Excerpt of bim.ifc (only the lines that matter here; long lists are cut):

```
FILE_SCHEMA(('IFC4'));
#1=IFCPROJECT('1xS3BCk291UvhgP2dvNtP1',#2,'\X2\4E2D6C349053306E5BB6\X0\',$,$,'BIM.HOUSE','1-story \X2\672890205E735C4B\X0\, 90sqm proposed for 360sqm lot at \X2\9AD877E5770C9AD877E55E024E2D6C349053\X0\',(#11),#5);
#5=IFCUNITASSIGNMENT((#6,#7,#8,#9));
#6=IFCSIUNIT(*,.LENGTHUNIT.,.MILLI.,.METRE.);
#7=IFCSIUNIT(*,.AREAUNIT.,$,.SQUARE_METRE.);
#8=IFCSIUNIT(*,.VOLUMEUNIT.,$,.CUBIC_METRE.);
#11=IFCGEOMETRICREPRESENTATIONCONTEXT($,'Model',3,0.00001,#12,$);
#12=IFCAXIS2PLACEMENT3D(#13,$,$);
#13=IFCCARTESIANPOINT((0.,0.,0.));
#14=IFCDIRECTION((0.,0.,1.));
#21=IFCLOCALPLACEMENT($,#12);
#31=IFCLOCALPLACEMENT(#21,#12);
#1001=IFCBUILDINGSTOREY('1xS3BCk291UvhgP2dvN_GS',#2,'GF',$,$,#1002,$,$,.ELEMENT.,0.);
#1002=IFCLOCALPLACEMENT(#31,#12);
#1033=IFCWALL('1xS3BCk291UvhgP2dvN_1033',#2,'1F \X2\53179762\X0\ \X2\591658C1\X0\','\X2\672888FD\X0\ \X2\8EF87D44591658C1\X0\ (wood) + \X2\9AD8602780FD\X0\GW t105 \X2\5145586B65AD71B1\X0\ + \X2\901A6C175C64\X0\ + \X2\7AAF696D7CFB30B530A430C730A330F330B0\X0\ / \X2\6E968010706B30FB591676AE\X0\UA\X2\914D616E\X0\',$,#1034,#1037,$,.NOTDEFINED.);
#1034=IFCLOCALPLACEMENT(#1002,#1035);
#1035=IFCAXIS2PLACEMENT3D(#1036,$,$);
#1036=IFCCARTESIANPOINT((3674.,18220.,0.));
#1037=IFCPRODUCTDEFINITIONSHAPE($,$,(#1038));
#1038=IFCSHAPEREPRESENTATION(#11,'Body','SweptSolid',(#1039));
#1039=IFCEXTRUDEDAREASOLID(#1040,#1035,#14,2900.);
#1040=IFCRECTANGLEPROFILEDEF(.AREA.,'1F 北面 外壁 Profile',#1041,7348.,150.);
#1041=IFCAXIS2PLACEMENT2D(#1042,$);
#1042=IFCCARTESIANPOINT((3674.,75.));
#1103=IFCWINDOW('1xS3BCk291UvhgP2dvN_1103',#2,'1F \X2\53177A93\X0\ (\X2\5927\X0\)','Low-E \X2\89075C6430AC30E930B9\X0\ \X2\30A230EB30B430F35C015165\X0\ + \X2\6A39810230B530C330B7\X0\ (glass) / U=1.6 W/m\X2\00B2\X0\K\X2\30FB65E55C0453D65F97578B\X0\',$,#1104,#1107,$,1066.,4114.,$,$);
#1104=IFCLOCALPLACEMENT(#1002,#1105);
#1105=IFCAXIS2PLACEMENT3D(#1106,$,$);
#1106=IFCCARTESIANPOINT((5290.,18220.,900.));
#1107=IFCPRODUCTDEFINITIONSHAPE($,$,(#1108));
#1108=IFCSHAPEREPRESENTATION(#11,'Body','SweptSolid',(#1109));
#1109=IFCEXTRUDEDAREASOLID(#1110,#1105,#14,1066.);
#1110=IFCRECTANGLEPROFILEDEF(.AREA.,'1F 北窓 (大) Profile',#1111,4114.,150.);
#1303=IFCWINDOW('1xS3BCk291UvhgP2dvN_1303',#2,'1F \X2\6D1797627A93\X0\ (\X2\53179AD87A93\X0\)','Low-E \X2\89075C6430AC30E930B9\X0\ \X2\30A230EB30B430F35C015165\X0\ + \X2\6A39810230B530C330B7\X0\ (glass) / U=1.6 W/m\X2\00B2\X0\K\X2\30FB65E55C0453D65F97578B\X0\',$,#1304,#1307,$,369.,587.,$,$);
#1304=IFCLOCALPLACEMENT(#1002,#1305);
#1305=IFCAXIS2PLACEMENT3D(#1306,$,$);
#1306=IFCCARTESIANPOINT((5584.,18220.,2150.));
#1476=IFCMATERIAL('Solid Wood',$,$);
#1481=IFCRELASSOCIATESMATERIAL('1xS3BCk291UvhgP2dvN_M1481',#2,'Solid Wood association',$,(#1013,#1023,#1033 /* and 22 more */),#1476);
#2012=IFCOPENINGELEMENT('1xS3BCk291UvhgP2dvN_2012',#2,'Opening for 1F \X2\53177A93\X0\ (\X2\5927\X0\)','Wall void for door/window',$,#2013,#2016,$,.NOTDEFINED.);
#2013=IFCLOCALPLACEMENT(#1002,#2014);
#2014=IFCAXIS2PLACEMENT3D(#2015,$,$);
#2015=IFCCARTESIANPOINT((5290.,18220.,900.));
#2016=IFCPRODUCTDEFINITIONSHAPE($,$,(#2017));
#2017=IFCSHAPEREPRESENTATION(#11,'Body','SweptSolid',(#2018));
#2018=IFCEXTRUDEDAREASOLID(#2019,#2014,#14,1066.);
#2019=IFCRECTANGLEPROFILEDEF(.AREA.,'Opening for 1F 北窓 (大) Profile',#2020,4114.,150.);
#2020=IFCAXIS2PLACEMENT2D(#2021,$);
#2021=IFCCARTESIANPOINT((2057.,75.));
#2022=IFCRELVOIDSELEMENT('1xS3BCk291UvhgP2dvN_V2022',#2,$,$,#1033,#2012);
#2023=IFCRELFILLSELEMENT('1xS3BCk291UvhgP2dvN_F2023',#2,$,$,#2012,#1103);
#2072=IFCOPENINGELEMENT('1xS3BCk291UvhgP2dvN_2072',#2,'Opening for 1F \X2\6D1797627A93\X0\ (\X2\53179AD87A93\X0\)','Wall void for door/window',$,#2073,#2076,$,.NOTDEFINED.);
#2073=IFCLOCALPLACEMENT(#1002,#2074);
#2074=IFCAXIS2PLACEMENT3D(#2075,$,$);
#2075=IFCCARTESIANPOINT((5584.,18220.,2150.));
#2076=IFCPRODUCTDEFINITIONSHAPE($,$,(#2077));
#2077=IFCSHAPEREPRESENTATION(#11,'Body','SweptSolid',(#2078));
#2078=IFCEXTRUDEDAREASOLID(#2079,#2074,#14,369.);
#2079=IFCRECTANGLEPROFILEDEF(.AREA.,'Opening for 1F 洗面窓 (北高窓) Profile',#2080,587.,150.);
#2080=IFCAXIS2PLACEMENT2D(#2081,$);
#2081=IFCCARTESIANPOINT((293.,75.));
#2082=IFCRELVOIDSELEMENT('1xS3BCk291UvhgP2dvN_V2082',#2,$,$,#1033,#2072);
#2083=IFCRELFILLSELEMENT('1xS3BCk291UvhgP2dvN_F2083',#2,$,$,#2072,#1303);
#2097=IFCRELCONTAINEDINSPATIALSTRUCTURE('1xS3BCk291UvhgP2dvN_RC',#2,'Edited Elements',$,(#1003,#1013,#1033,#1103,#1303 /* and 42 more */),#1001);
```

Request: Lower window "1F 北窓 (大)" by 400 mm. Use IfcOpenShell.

```python
import numpy as np
import ifcopenshell
import ifcopenshell.api.geometry
import ifcopenshell.util.placement
import ifcopenshell.util.unit

model = ifcopenshell.open("bim.ifc")
unit_scale = ifcopenshell.util.unit.calculate_unit_scale(model)

window = model.by_guid("1xS3BCk291UvhgP2dvN_1103")
opening = window.FillsVoids[0].RelatingOpeningElement
dz = -400.0

shift = np.array([0.0, 0.0, dz])
# The window is not placed relative to its opening, so move both.
for product in (opening, window):
    matrix = ifcopenshell.util.placement.get_local_placement(product.ObjectPlacement)
    matrix[:3, 3] += shift
    ifcopenshell.api.geometry.edit_object_placement(model, product=product, matrix=matrix, is_si=False)

print(f"moved by {dz * unit_scale:+.3f} m")

model.write("bim_edited.ifc")
```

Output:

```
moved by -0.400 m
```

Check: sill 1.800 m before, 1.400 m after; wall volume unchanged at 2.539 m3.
